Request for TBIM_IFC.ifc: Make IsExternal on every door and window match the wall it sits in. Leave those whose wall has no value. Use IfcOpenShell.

First a look at what the model holds.

```python
import ifcopenshell
import ifcopenshell.util.element

model = ifcopenshell.open("TBIM_IFC.ifc")
print(model.schema)
seen = {}
for e in model.by_type("IfcDoor") + model.by_type("IfcWindow"):
    if not e.FillsVoids:
        continue
    host = e.FillsVoids[0].RelatingOpeningElement.VoidsElements[0].RelatingBuildingElement
    own = ifcopenshell.util.element.get_pset(e, f"Pset_{e.is_a()[3:].removesuffix('StandardCase')}Common", "IsExternal")
    wall = ifcopenshell.util.element.get_pset(host, "Pset_WallCommon", "IsExternal")
    seen[e.is_a(), own, wall] = seen.get((e.is_a(), own, wall), 0) + 1
for (cls, own, wall), count in sorted(seen.items(), key=str):
    print(count, cls, "IsExternal:", own, "| host wall:", wall)
```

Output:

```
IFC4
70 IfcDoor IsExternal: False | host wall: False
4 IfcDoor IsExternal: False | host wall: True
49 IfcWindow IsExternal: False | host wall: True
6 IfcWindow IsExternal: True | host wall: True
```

```python
import ifcopenshell
import ifcopenshell.api.pset
import ifcopenshell.util.element

model = ifcopenshell.open("TBIM_IFC.ifc")

count = 0
for ifc_class, pset_name in (("IfcDoor", "Pset_DoorCommon"), ("IfcWindow", "Pset_WindowCommon")):
    for e in model.by_type(ifc_class):
        if not e.FillsVoids:
            continue
        host = e.FillsVoids[0].RelatingOpeningElement.VoidsElements[0].RelatingBuildingElement
        external = ifcopenshell.util.element.get_pset(host, "Pset_WallCommon", "IsExternal")
        if external is None or ifcopenshell.util.element.get_pset(e, pset_name, "IsExternal") == external:
            continue
        pset = ifcopenshell.api.pset.add_pset(model, product=e, name=pset_name)
        ifcopenshell.api.pset.edit_pset(model, pset=pset, properties={"IsExternal": external})
        count += 1

print(count, "updated")

model.write("TBIM_IFC_rev.ifc")
```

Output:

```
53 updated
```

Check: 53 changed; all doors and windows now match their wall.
